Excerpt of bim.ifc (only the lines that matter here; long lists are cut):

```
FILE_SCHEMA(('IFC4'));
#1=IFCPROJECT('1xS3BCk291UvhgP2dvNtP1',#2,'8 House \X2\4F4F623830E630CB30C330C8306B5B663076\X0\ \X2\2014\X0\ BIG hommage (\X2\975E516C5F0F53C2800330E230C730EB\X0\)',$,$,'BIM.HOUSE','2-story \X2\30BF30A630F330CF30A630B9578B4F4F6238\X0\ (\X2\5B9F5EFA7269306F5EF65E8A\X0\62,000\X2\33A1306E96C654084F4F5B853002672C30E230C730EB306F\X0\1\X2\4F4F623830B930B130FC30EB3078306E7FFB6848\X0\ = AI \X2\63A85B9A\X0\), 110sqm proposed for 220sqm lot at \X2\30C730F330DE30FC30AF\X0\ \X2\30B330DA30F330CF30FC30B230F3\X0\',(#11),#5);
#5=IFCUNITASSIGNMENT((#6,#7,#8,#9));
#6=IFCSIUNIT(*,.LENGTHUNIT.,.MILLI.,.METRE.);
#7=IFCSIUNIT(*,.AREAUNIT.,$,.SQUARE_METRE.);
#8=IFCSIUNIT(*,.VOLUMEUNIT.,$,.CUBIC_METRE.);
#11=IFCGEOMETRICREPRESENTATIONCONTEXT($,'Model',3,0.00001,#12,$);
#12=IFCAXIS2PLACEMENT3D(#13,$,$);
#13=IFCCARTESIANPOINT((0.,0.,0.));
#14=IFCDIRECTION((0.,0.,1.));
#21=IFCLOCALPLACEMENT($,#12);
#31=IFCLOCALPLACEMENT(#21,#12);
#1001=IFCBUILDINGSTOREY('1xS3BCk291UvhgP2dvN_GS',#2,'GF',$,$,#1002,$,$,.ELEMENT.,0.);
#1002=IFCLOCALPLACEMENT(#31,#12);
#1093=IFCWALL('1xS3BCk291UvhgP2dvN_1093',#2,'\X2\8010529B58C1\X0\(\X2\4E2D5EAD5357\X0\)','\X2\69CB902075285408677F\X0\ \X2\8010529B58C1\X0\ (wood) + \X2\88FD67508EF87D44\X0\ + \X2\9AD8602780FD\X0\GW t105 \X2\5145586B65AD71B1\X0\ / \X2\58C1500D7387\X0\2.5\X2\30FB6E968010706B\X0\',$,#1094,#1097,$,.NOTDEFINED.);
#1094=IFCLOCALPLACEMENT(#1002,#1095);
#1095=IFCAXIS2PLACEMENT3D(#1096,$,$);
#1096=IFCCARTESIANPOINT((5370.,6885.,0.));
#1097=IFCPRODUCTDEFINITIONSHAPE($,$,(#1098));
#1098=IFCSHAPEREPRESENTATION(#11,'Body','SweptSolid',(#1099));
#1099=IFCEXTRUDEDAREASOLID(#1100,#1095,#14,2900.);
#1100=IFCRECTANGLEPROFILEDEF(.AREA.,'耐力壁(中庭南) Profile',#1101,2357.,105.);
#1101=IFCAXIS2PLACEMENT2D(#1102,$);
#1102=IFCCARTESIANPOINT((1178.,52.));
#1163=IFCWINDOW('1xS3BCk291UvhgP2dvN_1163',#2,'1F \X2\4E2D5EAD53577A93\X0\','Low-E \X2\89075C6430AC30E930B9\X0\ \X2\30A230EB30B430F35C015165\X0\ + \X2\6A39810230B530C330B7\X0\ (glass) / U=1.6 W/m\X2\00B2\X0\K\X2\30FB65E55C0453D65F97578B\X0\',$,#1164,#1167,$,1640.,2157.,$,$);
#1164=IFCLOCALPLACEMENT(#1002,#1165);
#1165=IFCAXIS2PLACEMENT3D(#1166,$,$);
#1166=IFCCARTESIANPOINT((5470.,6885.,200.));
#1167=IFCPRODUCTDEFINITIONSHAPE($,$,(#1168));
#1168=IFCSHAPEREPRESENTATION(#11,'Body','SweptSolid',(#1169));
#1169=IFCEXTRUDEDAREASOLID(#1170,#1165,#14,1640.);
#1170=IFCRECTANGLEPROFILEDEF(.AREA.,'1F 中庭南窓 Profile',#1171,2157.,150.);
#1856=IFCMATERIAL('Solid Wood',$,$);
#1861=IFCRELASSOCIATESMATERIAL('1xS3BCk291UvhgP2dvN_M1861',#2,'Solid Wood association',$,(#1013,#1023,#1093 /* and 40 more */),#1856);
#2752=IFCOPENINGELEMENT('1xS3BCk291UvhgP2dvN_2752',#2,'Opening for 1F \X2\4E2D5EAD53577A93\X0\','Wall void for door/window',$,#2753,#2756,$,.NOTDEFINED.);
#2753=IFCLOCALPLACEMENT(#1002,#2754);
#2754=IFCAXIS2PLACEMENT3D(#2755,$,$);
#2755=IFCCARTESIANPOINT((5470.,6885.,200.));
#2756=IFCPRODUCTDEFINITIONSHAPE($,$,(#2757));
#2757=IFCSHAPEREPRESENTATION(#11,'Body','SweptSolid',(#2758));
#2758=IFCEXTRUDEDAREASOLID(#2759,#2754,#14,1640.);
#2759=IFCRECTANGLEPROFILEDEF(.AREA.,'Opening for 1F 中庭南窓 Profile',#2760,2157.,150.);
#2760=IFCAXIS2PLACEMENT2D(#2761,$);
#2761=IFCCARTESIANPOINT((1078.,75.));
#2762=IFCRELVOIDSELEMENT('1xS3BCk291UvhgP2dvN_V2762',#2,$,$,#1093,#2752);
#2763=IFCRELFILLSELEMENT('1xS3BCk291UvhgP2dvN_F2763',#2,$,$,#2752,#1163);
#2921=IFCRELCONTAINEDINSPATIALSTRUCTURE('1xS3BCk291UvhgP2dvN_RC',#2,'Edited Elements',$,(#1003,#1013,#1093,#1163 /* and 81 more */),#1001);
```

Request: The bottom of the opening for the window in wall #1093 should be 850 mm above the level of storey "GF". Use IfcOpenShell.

```python
import numpy as np
import ifcopenshell
import ifcopenshell.api.geometry
import ifcopenshell.geom
import ifcopenshell.util.element
import ifcopenshell.util.placement
import ifcopenshell.util.shape
import ifcopenshell.util.unit

model = ifcopenshell.open("bim.ifc")
unit_scale = ifcopenshell.util.unit.calculate_unit_scale(model)

window = model.by_guid("1xS3BCk291UvhgP2dvN_1163")
opening = window.FillsVoids[0].RelatingOpeningElement
storey = ifcopenshell.util.element.get_container(window, ifc_class="IfcBuildingStorey")
level = ifcopenshell.util.placement.get_local_placement(storey.ObjectPlacement)[2, 3]

# The opening's origin need not be at the sill, so measure its lowest point.
shape = ifcopenshell.geom.create_shape(ifcopenshell.geom.settings(), opening)
bottom = ifcopenshell.util.shape.get_shape_bottom_elevation(shape, shape.geometry) / unit_scale
dz = level + 0.85 / unit_scale - bottom

shift = np.array([0.0, 0.0, dz])
# The window is not placed relative to its opening, so move both.
for product in (opening, window):
    matrix = ifcopenshell.util.placement.get_local_placement(product.ObjectPlacement)
    matrix[:3, 3] += shift
    ifcopenshell.api.geometry.edit_object_placement(model, product=product, matrix=matrix, is_si=False)

print(f"moved by {dz * unit_scale:+.3f} m")

model.write("bim_edited.ifc")
```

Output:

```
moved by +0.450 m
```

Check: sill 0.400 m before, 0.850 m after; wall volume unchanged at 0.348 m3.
